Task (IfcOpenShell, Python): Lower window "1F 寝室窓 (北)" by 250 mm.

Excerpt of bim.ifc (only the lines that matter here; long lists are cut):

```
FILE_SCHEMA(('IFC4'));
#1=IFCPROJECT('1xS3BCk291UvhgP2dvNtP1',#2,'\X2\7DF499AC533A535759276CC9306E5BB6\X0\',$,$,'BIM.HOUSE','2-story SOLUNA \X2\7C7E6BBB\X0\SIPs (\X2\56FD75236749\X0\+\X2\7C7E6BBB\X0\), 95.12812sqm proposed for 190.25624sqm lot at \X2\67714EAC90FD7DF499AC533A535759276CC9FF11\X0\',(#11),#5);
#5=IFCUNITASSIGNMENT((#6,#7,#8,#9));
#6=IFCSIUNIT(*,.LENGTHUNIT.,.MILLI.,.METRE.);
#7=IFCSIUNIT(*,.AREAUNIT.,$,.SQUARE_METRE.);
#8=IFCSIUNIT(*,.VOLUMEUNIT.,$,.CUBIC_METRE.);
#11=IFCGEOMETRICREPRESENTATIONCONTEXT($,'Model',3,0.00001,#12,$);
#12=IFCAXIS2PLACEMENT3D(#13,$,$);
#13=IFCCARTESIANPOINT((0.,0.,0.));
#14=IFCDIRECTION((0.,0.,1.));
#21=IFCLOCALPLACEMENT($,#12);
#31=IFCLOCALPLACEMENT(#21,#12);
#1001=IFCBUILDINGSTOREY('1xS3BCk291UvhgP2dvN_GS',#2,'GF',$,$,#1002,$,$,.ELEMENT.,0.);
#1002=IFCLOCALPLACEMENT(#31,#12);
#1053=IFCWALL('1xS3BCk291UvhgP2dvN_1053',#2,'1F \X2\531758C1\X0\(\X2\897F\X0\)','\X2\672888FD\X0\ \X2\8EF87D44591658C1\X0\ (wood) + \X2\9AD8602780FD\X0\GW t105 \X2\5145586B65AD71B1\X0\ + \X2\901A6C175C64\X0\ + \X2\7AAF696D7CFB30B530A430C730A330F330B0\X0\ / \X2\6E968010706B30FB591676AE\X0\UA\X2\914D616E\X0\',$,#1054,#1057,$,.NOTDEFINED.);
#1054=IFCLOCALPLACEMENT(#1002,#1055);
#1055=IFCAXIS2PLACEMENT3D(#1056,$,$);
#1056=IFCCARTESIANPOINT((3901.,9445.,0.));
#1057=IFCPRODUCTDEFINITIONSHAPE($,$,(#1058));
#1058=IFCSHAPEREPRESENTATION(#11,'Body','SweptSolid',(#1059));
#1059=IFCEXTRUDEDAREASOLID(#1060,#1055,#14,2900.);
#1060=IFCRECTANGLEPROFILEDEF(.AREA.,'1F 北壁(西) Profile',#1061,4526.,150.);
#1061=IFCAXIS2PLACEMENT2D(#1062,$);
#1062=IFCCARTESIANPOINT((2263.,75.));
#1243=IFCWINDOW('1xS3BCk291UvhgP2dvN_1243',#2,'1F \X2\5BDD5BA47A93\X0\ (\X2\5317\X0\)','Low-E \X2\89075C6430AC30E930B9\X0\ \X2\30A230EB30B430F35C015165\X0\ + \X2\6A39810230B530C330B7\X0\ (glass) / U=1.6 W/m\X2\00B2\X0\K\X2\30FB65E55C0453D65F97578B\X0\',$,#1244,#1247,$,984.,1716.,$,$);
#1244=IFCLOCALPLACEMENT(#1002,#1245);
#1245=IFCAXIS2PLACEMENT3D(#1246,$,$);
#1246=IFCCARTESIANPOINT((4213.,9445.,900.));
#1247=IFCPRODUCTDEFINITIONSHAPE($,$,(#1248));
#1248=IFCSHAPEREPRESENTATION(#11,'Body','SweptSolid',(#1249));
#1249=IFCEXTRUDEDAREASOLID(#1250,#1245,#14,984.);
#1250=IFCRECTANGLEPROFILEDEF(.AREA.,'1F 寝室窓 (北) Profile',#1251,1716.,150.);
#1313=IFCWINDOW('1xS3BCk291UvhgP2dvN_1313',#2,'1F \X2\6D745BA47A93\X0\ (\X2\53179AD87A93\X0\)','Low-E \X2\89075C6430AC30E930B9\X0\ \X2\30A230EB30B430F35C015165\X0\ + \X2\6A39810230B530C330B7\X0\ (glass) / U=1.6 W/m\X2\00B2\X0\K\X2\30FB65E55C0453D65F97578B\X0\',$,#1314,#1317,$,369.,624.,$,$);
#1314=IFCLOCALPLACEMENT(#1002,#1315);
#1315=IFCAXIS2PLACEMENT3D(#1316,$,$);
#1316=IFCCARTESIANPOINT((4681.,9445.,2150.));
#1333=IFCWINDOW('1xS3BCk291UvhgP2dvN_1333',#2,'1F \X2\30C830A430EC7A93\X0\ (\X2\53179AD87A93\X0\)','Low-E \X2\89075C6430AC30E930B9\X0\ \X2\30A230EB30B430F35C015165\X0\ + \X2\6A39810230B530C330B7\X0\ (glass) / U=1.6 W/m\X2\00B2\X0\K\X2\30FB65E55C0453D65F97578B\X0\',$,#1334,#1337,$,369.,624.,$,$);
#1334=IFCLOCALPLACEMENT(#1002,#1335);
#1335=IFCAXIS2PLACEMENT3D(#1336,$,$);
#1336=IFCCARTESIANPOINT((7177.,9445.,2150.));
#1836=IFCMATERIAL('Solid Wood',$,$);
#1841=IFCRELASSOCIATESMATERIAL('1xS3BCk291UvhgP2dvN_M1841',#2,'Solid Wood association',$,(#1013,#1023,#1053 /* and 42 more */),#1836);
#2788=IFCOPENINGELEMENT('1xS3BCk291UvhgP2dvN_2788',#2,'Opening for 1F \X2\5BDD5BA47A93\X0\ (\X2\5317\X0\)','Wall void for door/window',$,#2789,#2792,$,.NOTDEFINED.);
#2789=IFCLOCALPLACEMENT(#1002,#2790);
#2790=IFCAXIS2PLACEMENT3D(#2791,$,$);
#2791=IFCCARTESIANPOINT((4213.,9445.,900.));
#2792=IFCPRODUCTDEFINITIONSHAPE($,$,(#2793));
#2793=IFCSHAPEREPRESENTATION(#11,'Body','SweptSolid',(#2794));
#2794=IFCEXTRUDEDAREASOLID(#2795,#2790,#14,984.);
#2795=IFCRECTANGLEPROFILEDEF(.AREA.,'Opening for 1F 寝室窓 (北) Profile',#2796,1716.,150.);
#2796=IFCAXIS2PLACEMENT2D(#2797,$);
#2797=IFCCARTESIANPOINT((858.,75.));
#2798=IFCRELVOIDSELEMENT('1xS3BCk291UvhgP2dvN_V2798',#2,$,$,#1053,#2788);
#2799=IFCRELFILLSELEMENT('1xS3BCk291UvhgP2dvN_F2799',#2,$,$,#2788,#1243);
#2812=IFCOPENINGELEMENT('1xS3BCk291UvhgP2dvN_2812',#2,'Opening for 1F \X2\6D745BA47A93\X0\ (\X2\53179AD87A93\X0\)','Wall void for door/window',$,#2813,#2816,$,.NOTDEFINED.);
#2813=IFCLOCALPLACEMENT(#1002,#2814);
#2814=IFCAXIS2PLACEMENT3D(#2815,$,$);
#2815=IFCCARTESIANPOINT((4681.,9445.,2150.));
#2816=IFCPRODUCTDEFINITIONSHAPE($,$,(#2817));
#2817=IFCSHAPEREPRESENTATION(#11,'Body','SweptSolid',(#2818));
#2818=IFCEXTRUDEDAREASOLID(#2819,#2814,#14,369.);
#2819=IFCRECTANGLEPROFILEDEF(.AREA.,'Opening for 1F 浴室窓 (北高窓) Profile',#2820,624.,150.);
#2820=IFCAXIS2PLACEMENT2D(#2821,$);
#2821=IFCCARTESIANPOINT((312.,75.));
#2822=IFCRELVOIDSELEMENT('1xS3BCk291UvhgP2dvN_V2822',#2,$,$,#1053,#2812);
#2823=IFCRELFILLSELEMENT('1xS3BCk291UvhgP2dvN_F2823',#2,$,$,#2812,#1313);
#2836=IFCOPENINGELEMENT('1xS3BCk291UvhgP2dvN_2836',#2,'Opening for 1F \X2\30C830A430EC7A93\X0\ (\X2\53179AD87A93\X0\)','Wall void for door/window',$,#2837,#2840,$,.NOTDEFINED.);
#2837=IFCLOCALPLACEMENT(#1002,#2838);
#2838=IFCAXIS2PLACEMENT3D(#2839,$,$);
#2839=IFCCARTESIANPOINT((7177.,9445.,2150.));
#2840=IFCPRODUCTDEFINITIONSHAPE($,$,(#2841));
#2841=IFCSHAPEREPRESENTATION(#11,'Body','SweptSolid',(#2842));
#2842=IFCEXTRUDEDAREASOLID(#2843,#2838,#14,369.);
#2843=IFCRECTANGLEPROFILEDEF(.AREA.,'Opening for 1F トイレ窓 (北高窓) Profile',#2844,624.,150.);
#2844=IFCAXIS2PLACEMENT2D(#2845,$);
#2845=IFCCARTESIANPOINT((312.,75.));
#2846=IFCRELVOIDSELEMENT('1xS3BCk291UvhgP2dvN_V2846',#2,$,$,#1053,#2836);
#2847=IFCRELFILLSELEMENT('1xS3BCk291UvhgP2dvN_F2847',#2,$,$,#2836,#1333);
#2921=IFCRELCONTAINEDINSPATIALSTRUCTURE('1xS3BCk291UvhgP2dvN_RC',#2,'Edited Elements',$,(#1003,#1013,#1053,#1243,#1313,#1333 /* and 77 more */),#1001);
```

```python
import numpy as np
import ifcopenshell
import ifcopenshell.api.geometry
import ifcopenshell.util.placement
import ifcopenshell.util.unit

model = ifcopenshell.open("bim.ifc")
unit_scale = ifcopenshell.util.unit.calculate_unit_scale(model)

window = model.by_id(1243)
opening = window.FillsVoids[0].RelatingOpeningElement
dz = -0.25 / unit_scale

shift = np.array([0.0, 0.0, dz])
# The window is not placed relative to its opening, so move both.
for product in (opening, window):
    matrix = ifcopenshell.util.placement.get_local_placement(product.ObjectPlacement)
    matrix[:3, 3] += shift
    ifcopenshell.api.geometry.edit_object_placement(model, product=product, matrix=matrix, is_si=False)

print(f"moved by {dz * unit_scale:+.3f} m")

model.write("bim_edited.ifc")
```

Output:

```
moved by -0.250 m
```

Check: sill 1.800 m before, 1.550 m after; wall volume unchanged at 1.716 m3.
